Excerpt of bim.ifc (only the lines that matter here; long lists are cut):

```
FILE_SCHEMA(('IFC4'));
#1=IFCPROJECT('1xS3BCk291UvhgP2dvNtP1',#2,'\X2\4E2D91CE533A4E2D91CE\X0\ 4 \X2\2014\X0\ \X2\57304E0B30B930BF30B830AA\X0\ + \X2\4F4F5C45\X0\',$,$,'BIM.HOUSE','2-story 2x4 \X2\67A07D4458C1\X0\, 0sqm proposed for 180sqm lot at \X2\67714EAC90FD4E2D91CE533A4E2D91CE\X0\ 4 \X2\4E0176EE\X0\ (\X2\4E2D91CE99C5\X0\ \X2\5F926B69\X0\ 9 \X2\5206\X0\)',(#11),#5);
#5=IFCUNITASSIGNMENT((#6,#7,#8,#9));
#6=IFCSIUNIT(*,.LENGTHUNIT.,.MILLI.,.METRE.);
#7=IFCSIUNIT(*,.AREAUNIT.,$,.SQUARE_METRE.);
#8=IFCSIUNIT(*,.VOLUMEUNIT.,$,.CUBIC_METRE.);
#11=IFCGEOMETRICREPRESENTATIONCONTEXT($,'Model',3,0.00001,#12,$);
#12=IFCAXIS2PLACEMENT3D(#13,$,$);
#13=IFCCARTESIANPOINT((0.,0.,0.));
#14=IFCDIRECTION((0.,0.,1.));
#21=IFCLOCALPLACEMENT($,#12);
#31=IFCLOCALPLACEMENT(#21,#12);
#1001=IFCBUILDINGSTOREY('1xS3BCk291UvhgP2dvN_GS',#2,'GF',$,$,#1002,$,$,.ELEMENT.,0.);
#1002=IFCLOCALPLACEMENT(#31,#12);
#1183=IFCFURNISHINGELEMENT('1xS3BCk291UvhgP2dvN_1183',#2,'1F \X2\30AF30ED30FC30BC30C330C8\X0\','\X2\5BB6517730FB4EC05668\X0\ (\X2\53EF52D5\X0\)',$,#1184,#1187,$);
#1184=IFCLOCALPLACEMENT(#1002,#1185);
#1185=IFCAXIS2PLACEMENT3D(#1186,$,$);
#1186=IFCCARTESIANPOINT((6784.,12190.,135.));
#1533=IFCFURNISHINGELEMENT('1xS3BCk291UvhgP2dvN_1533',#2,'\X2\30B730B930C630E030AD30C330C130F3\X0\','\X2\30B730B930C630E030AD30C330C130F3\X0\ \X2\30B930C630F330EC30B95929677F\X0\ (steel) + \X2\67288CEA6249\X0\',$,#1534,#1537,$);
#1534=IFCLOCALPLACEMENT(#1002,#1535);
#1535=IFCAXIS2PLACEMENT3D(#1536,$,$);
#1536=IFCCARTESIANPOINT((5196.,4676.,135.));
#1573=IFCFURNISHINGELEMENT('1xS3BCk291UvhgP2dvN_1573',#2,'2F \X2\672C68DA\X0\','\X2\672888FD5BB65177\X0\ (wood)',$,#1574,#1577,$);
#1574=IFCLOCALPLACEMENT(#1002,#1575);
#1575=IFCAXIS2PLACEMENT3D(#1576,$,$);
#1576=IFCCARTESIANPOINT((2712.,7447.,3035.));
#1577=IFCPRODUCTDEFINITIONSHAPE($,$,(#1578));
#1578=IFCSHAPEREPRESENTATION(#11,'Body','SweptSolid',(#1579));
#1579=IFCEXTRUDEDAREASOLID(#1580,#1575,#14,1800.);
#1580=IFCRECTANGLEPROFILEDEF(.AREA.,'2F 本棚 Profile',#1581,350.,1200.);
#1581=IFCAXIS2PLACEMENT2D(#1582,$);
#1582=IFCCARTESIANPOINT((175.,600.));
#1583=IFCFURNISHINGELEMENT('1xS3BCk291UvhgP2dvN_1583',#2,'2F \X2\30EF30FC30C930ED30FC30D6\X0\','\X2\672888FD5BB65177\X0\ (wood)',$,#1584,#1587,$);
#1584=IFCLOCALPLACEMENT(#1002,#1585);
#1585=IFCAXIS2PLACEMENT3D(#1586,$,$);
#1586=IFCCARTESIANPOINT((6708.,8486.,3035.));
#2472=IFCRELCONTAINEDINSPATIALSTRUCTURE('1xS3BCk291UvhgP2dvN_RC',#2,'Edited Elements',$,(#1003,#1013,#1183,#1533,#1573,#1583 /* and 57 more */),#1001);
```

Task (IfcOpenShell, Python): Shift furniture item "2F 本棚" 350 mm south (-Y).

```python
import ifcopenshell
import ifcopenshell.api.geometry
import ifcopenshell.util.placement

model = ifcopenshell.open("bim.ifc")

item = model.by_id(1573)
matrix = ifcopenshell.util.placement.get_local_placement(item.ObjectPlacement)
matrix[1, 3] -= 350.0
ifcopenshell.api.geometry.edit_object_placement(model, product=item, matrix=matrix, is_si=False)

print(ifcopenshell.util.placement.get_local_placement(item.ObjectPlacement).round(3) + 0.0)

model.write("bim-out.ifc")
```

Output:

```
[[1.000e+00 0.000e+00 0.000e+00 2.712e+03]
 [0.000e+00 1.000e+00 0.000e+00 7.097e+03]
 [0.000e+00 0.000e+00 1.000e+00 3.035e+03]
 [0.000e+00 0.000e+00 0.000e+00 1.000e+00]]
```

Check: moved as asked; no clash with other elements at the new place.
